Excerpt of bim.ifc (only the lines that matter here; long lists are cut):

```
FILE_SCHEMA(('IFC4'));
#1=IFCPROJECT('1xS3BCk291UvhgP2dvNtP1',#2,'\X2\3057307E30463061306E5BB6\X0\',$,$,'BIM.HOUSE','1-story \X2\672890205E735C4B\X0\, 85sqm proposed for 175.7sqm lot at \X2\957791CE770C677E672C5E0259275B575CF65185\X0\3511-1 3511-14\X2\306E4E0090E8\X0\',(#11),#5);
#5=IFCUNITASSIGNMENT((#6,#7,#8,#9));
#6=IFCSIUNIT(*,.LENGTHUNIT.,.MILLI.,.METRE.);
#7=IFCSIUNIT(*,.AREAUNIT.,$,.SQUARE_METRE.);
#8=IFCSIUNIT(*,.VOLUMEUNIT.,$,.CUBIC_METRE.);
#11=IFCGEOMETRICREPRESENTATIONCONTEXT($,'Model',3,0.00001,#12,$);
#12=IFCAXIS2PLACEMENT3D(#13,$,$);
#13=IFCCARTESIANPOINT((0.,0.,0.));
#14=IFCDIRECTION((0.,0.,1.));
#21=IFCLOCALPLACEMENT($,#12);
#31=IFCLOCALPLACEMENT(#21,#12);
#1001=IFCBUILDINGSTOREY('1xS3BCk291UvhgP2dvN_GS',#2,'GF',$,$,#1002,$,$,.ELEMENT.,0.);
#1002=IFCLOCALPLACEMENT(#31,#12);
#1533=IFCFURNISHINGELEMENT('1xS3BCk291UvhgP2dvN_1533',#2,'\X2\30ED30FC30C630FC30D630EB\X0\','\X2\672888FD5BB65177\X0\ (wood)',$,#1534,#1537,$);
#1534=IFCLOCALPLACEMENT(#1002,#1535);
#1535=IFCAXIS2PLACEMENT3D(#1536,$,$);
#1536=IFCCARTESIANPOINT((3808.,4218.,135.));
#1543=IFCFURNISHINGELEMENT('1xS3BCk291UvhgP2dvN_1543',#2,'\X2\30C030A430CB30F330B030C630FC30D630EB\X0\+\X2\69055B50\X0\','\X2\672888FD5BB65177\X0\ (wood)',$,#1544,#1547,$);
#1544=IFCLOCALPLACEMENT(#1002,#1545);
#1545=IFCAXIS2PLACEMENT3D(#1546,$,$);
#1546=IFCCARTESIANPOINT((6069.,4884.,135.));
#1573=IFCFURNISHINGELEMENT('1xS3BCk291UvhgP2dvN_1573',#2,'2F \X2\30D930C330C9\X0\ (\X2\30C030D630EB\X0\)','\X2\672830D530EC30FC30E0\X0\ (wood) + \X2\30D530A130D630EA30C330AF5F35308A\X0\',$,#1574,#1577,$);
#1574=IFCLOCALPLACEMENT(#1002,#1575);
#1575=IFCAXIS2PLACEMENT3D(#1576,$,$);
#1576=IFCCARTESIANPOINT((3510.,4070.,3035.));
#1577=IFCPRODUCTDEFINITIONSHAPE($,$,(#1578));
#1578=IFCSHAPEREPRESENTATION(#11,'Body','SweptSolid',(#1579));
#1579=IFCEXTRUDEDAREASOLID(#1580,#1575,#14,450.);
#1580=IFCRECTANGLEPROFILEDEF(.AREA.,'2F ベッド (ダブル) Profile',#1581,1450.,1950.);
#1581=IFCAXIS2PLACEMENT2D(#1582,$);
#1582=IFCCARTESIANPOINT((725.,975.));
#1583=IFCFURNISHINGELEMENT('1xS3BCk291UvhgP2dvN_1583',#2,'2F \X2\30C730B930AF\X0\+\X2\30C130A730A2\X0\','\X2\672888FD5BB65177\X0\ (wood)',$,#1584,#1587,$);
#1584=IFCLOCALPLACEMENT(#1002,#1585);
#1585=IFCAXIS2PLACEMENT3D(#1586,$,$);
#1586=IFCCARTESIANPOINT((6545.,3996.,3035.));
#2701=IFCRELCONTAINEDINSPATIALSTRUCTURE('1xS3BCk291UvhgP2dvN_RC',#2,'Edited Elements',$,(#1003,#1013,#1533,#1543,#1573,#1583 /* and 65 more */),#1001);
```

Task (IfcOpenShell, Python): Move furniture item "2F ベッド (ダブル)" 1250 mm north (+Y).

```python
import ifcopenshell
import ifcopenshell.api.geometry
import ifcopenshell.util.placement
import ifcopenshell.util.unit

model = ifcopenshell.open("bim.ifc")
unit_scale = ifcopenshell.util.unit.calculate_unit_scale(model)

item = model.by_guid("1xS3BCk291UvhgP2dvN_1573")
matrix = ifcopenshell.util.placement.get_local_placement(item.ObjectPlacement)
matrix[1, 3] += 1.25 / unit_scale
ifcopenshell.api.geometry.edit_object_placement(model, product=item, matrix=matrix, is_si=False)

print(ifcopenshell.util.placement.get_local_placement(item.ObjectPlacement).round(3) + 0.0)

model.write("bim_edited.ifc")
```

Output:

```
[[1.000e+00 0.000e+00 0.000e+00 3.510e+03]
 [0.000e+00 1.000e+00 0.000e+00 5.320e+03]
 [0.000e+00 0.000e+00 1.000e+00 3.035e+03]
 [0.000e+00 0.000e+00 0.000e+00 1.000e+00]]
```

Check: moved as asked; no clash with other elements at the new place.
